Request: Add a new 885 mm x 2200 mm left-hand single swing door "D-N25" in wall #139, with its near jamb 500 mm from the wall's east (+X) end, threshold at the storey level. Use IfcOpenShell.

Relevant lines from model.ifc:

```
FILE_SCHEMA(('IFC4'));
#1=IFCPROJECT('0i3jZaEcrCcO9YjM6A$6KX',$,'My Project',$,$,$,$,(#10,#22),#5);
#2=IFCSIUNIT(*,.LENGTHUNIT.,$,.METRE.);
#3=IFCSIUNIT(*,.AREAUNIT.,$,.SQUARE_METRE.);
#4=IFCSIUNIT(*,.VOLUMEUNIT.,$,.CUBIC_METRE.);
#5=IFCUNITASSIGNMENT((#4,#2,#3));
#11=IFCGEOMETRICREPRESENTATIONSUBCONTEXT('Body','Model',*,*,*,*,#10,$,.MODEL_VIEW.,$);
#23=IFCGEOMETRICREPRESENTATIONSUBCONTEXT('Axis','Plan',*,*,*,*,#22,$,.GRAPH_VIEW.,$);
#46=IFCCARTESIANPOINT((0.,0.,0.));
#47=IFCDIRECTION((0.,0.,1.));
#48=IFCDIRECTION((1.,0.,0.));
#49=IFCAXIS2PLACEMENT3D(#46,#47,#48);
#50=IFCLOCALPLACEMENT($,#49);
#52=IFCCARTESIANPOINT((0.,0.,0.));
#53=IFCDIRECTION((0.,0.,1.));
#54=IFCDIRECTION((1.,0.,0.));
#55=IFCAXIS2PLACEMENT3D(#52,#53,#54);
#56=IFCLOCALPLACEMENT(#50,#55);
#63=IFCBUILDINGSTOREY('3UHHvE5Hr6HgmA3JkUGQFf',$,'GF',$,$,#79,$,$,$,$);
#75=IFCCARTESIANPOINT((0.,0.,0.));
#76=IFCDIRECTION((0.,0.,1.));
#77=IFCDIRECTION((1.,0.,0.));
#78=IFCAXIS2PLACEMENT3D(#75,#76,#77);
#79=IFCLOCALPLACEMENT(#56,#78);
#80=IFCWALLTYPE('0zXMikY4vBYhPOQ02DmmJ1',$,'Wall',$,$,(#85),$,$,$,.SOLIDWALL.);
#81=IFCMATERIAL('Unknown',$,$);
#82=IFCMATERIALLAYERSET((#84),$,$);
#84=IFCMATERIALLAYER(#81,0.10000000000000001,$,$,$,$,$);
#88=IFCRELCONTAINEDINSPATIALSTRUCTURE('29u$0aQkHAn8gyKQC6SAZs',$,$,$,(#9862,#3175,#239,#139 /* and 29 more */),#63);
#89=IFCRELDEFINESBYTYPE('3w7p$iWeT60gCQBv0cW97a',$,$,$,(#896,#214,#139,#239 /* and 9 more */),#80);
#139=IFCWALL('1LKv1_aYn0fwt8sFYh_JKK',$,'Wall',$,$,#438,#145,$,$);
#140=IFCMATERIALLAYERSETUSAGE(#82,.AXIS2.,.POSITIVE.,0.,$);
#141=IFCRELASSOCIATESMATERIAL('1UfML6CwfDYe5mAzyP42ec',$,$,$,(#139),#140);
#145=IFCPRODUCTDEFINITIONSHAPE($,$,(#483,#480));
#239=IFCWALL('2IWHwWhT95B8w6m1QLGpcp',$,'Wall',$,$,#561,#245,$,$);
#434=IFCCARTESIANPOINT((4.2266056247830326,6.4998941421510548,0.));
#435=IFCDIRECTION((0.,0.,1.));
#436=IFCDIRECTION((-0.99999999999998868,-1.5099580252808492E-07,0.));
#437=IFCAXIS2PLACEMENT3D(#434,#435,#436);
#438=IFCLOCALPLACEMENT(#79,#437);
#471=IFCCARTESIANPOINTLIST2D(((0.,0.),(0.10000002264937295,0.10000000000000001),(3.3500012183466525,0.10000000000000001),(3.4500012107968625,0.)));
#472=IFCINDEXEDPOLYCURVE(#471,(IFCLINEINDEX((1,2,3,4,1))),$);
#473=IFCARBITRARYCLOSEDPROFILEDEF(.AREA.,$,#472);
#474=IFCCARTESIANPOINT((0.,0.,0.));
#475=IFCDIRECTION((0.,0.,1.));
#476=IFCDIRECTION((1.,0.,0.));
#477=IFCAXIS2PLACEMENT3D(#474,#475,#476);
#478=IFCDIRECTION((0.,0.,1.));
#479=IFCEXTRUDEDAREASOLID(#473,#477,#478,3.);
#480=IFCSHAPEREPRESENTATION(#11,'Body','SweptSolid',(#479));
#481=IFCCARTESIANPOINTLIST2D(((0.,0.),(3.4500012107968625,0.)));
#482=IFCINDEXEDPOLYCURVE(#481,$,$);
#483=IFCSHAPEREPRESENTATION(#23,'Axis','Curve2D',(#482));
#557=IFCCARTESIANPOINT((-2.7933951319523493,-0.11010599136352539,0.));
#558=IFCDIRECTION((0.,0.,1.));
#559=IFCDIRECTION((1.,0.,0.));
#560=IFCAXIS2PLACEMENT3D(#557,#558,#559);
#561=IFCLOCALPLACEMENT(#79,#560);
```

```python
import numpy as np
import ifcopenshell
import ifcopenshell.api.feature
import ifcopenshell.api.geometry
import ifcopenshell.api.root
import ifcopenshell.api.spatial
import ifcopenshell.geom
import ifcopenshell.util.element
import ifcopenshell.util.placement
import ifcopenshell.util.representation
import ifcopenshell.util.shape
import ifcopenshell.util.unit

model = ifcopenshell.open("model.ifc")
unit_scale = ifcopenshell.util.unit.calculate_unit_scale(model)
settings = ifcopenshell.geom.settings()


def volume(element):
    """Net volume in cubic metres, openings subtracted."""
    shape = ifcopenshell.geom.create_shape(settings, element)
    return ifcopenshell.util.shape.get_volume(shape.geometry)


wall = model.by_id(139)
storey = ifcopenshell.util.element.get_container(wall, ifc_class="IfcBuildingStorey")
context = ifcopenshell.util.representation.get_context(model, "Model", "Body", "MODEL_VIEW")
before = volume(wall)

width, height, from_end, sill = 0.885, 2.2, 0.5, 0.0  # metres

# The wall runs along its own X axis, and the end named is its -X end.
wall_shape = ifcopenshell.geom.create_shape(settings, wall)
x, y, z = ifcopenshell.util.shape.get_vertices(wall_shape.geometry).T
start = x.min() + from_end
face, thickness = float(y.min()), float(y.max() - y.min())
wall_matrix = ifcopenshell.util.placement.get_local_placement(wall.ObjectPlacement)
level = ifcopenshell.util.placement.get_local_placement(storey.ObjectPlacement)[2, 3]


def in_wall(x, y):
    """Placement at x, y metres in the wall's axes, at sill height."""
    matrix = wall_matrix.copy()
    matrix[:, 3] = wall_matrix @ np.array([x / unit_scale, y / unit_scale, 0.0, 1.0])
    matrix[2, 3] = level + sill / unit_scale
    return matrix


# Opening: a box that overshoots both wall faces by 50 mm.
opening = ifcopenshell.api.root.create_entity(model, ifc_class="IfcOpeningElement", predefined_type="OPENING")
box = ifcopenshell.api.geometry.add_wall_representation(
    model, context=context, length=width, height=height, thickness=thickness + 0.1
)
ifcopenshell.api.geometry.assign_representation(model, product=opening, representation=box)
ifcopenshell.api.geometry.edit_object_placement(model, product=opening, matrix=in_wall(start, face - 0.05), is_si=False)
ifcopenshell.api.feature.add_feature(model, feature=opening, element=wall)

door = ifcopenshell.api.root.create_entity(model, ifc_class="IfcDoor", name="D-N25", predefined_type="DOOR")
door.OverallWidth, door.OverallHeight = width / unit_scale, height / unit_scale
door.OperationType = "SINGLE_SWING_LEFT"
body = ifcopenshell.api.geometry.add_door_representation(
    model,
    context=context,
    overall_width=door.OverallWidth,
    overall_height=door.OverallHeight,
    operation_type="SINGLE_SWING_LEFT",
    lining_properties={"LiningDepth": thickness / unit_scale, "ThresholdDepth": thickness / unit_scale},
)
ifcopenshell.api.geometry.assign_representation(model, product=door, representation=body)
ifcopenshell.api.spatial.assign_container(model, products=[door], relating_structure=storey)
ifcopenshell.api.feature.add_filling(model, opening=opening, element=door)

# The lining spans the wall, so the door starts at the wall face.
ifcopenshell.api.geometry.edit_object_placement(model, product=door, matrix=in_wall(start, face), is_si=False)

after = volume(wall)

print(f"wall volume {before:.3f} -> {after:.3f} m3")

model.write("model_v2.ifc")
```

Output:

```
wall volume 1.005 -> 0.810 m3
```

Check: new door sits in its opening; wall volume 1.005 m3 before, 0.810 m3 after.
